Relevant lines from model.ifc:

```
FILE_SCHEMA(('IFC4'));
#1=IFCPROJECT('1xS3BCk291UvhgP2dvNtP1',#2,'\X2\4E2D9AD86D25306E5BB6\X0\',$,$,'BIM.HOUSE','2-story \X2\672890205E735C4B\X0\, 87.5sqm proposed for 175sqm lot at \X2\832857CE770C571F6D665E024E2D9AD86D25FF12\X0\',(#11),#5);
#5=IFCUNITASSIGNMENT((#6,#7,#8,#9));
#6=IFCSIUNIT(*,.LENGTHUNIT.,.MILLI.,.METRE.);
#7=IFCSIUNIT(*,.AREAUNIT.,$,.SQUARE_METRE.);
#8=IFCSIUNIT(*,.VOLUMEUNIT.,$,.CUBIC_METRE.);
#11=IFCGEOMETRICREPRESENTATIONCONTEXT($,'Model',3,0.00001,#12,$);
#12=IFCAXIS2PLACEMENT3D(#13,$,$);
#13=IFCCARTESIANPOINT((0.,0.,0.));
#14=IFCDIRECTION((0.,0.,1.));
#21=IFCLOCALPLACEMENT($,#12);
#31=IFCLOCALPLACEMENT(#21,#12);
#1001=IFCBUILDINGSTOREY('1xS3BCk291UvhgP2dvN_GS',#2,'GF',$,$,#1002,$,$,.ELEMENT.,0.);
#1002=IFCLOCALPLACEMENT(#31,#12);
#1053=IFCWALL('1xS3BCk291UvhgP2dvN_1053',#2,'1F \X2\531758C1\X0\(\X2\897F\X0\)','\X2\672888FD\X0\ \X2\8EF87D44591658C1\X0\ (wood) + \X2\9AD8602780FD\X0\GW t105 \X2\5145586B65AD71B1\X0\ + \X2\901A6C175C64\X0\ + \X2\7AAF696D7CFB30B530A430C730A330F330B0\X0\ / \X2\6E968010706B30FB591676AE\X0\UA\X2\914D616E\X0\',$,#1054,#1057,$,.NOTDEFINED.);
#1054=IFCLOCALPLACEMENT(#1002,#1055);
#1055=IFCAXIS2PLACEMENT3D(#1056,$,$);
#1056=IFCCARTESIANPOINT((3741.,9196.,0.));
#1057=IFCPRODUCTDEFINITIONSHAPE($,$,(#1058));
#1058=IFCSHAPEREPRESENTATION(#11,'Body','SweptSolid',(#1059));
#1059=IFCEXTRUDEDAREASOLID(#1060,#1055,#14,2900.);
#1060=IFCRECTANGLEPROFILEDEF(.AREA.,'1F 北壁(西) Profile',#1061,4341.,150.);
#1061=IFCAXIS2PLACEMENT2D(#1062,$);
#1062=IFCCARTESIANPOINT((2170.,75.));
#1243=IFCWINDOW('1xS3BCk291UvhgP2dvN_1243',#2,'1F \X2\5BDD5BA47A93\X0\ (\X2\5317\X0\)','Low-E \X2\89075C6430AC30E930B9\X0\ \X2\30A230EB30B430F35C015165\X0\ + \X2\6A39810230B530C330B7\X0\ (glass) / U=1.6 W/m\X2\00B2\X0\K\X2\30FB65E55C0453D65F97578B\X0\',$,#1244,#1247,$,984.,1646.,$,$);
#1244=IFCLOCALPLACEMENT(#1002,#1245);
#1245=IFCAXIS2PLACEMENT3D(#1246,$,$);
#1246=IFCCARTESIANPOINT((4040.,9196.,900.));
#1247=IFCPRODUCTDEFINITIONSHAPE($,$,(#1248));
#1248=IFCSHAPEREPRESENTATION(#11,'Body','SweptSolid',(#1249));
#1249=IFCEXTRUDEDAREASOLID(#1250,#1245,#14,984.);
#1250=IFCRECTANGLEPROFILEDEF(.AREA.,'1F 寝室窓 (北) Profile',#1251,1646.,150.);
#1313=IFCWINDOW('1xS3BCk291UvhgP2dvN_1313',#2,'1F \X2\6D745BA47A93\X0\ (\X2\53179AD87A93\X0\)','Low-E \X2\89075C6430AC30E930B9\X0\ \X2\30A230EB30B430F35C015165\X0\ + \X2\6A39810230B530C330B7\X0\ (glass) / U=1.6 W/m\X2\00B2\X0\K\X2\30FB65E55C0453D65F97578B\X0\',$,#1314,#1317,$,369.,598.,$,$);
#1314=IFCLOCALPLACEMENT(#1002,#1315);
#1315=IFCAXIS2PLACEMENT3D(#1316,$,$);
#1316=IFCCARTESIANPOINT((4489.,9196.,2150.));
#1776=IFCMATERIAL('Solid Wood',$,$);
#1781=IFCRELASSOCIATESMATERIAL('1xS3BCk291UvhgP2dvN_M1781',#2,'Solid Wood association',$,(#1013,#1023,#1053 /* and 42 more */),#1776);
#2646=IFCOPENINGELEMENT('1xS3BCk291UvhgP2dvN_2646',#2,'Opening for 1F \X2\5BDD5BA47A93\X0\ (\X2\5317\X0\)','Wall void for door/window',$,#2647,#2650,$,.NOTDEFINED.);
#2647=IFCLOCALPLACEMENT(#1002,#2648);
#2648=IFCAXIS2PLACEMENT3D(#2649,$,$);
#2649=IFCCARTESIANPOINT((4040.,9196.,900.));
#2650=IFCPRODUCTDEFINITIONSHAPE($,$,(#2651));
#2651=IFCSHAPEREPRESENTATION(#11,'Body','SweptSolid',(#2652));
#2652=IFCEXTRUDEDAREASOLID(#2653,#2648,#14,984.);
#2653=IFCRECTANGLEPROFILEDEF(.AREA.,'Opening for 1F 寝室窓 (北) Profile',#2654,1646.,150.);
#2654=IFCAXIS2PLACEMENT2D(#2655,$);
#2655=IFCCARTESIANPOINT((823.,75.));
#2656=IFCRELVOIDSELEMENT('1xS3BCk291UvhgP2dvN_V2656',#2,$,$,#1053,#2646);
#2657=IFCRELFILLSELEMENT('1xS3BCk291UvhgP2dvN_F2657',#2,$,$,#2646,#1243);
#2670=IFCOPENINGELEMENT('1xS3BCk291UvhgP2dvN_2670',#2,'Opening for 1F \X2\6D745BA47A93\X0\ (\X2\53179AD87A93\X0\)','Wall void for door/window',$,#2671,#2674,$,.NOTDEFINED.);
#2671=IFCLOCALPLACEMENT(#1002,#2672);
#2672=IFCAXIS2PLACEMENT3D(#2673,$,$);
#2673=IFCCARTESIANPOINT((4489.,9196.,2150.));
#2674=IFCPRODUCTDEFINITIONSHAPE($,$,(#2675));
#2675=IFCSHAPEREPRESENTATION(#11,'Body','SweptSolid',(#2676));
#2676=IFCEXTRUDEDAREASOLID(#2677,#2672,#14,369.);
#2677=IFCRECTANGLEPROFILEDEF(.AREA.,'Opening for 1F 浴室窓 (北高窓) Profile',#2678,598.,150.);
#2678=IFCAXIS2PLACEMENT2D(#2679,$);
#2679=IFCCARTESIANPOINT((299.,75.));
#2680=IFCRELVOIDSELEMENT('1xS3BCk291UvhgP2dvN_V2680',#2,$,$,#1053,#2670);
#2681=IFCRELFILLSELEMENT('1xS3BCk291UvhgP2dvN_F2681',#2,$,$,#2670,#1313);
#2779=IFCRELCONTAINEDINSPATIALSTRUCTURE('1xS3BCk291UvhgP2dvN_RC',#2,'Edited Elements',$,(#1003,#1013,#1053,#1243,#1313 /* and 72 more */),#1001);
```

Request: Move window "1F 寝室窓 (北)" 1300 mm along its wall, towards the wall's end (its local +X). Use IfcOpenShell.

```python
import ifcopenshell
import ifcopenshell.api.geometry
import ifcopenshell.util.placement
import ifcopenshell.util.unit

model = ifcopenshell.open("model.ifc")
unit_scale = ifcopenshell.util.unit.calculate_unit_scale(model)

window = model.by_guid("1xS3BCk291UvhgP2dvN_1243")
opening = window.FillsVoids[0].RelatingOpeningElement
wall = opening.VoidsElements[0].RelatingBuildingElement

wall_matrix = ifcopenshell.util.placement.get_local_placement(wall.ObjectPlacement)
shift = wall_matrix[:3, 0] * 1.3 / unit_scale
before = ifcopenshell.util.placement.get_local_placement(window.ObjectPlacement)[:3, 3].copy()

# The window is not placed relative to its opening, so move both.
for product in (opening, window):
    matrix = ifcopenshell.util.placement.get_local_placement(product.ObjectPlacement)
    matrix[:3, 3] += shift
    ifcopenshell.api.geometry.edit_object_placement(model, product=product, matrix=matrix, is_si=False)

after = ifcopenshell.util.placement.get_local_placement(window.ObjectPlacement)[:3, 3]
print("window moved by", (after - before).round(3) + 0.0)

model.write("model_edited.ifc")
```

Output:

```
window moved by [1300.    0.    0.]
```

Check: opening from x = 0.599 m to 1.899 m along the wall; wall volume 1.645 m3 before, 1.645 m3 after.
